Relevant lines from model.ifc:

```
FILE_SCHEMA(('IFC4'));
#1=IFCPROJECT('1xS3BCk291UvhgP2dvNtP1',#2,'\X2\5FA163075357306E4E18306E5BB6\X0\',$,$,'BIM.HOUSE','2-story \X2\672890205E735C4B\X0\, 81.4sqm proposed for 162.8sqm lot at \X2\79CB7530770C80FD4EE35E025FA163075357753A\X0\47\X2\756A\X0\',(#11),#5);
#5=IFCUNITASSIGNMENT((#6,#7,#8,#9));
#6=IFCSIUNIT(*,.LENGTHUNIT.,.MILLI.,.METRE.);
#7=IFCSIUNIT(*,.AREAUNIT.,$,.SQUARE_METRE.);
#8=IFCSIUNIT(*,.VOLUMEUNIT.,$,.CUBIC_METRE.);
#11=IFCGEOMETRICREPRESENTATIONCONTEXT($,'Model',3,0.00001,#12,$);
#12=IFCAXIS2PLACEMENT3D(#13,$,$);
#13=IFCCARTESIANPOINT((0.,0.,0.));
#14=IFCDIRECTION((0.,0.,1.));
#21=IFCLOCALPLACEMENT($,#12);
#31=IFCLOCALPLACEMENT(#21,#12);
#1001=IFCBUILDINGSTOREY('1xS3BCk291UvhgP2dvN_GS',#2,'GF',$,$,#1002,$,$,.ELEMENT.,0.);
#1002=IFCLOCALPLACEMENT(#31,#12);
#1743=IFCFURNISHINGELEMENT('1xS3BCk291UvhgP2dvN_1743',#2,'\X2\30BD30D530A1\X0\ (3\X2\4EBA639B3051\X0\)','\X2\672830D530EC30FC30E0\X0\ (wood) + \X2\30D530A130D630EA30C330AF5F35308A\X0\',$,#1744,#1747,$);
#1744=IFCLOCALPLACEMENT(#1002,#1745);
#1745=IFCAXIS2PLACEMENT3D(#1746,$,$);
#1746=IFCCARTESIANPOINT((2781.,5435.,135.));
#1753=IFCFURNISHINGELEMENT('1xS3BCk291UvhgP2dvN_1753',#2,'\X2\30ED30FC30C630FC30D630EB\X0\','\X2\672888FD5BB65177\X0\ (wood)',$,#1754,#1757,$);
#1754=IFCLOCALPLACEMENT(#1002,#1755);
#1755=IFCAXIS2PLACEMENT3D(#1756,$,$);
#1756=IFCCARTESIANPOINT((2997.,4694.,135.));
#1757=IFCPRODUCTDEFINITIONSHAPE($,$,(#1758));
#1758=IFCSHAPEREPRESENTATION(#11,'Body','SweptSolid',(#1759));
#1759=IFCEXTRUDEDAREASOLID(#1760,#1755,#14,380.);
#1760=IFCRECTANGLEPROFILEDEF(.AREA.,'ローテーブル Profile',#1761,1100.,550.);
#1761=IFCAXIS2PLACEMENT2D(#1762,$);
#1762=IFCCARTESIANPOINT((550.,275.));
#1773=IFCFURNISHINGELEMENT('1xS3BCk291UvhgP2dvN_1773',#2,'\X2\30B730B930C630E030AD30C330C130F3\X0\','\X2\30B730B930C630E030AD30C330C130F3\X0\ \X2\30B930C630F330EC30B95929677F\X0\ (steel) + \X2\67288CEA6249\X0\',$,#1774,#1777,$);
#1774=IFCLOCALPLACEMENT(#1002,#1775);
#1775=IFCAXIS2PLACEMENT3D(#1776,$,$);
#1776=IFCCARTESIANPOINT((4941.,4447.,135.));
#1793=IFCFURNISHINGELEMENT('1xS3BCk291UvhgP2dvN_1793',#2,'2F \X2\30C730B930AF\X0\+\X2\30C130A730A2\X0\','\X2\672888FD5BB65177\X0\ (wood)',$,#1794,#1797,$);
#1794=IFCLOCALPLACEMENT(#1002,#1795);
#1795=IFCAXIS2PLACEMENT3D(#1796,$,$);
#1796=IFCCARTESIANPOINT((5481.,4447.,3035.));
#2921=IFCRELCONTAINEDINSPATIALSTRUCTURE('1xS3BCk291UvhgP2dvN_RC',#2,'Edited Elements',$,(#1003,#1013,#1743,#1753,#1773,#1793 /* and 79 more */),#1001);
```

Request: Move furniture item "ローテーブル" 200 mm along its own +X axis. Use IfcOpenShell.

```python
import ifcopenshell
import ifcopenshell.api.geometry
import ifcopenshell.util.placement

model = ifcopenshell.open("model.ifc")

item = model.by_guid("1xS3BCk291UvhgP2dvN_1753")
matrix = ifcopenshell.util.placement.get_local_placement(item.ObjectPlacement)
matrix[:3, 3] += matrix[:3, 0] * 200.0
ifcopenshell.api.geometry.edit_object_placement(model, product=item, matrix=matrix, is_si=False)

print(ifcopenshell.util.placement.get_local_placement(item.ObjectPlacement).round(3) + 0.0)

model.write("model_edited.ifc")
```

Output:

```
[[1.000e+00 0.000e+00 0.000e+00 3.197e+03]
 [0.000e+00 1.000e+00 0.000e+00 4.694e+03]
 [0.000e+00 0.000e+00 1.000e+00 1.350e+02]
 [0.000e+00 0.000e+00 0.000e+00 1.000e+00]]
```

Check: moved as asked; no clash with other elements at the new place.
